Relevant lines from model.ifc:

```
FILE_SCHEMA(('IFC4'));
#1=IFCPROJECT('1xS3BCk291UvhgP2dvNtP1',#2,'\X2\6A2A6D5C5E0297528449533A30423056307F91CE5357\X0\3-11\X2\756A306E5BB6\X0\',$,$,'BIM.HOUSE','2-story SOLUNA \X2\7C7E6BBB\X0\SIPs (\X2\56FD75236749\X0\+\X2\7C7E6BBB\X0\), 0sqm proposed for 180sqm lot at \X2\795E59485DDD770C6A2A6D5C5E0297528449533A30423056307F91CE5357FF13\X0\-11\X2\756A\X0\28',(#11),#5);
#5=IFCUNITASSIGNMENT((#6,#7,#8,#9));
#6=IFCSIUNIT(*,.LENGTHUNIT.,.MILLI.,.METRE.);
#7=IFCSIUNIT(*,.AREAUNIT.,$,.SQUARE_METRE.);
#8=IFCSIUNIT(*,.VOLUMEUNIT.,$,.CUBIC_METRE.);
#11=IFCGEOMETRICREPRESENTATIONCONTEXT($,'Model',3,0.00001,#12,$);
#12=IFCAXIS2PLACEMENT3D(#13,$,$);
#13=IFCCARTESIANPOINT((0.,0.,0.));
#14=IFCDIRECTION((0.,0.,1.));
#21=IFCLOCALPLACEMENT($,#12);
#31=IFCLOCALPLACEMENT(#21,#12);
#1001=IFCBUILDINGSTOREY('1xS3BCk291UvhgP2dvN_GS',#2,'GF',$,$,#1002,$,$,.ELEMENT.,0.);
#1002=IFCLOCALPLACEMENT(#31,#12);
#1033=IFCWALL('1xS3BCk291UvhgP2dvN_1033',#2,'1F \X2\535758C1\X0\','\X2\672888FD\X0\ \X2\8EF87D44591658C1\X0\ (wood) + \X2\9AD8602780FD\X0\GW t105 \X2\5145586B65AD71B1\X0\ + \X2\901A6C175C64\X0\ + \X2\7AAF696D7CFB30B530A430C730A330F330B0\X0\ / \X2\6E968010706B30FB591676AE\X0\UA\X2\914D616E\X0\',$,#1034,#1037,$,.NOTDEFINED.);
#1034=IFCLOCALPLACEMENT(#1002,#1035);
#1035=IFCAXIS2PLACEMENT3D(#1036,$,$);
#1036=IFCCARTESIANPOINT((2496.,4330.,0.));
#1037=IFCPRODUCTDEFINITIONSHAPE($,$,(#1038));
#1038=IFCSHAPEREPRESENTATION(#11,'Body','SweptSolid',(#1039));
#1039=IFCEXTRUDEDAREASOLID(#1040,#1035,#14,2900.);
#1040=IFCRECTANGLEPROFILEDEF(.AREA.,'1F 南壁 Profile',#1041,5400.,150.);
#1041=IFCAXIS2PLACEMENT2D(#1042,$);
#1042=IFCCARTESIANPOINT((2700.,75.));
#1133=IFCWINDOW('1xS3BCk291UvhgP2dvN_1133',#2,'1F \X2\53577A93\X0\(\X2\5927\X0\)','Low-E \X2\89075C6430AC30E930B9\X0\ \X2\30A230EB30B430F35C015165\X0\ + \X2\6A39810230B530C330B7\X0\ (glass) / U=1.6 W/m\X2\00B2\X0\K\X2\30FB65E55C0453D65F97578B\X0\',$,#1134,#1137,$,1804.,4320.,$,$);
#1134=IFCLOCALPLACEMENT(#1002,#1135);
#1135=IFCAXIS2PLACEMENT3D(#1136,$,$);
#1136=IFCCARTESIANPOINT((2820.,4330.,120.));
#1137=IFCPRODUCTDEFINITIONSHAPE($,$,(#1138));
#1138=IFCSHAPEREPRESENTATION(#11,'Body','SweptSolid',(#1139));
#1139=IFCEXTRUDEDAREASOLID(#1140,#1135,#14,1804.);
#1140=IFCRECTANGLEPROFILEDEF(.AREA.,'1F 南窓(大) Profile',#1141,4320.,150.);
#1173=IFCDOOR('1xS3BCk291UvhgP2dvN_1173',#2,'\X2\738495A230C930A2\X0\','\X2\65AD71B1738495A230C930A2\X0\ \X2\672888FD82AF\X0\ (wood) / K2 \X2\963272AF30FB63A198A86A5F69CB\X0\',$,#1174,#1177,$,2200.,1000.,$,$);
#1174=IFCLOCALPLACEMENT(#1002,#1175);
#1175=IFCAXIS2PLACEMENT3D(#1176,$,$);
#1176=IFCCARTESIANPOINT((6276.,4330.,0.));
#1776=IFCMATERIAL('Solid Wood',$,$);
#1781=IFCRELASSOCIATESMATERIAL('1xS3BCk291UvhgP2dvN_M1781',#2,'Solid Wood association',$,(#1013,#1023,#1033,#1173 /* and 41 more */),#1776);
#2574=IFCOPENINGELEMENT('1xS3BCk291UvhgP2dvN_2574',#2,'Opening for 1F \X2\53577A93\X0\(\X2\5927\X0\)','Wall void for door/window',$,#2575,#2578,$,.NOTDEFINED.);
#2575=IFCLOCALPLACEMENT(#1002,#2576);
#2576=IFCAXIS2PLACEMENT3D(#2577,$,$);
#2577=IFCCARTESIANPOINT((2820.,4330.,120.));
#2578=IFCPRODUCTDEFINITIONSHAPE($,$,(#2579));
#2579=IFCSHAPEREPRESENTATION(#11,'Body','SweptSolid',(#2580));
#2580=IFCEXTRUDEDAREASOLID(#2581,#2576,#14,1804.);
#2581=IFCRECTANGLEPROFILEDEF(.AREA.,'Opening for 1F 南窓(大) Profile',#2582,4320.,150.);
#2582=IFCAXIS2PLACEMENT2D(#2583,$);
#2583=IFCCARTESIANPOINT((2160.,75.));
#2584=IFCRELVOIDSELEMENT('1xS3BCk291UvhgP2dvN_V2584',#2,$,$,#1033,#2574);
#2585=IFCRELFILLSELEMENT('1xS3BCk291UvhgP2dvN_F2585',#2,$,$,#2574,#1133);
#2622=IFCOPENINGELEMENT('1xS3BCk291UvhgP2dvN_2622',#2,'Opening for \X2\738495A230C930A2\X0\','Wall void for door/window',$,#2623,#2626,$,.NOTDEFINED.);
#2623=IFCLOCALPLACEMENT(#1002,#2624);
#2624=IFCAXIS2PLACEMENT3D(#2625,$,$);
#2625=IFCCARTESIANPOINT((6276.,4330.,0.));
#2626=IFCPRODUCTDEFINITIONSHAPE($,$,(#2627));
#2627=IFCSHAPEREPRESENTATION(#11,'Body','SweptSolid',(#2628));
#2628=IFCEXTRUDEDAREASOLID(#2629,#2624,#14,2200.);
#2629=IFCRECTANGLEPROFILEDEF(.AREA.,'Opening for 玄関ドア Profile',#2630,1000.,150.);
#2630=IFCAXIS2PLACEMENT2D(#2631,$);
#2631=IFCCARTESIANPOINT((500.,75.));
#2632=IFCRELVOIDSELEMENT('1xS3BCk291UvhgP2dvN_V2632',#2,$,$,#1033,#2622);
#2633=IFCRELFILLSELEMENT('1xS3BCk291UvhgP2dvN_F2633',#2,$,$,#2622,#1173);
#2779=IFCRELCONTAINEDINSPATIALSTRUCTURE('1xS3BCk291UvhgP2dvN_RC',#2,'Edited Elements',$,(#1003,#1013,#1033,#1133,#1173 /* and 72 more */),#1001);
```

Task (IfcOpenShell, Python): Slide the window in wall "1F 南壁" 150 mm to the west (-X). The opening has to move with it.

```python
import ifcopenshell
import ifcopenshell.api.geometry
import ifcopenshell.util.placement
import ifcopenshell.util.unit

model = ifcopenshell.open("model.ifc")
unit_scale = ifcopenshell.util.unit.calculate_unit_scale(model)

window = model.by_guid("1xS3BCk291UvhgP2dvN_1133")
opening = window.FillsVoids[0].RelatingOpeningElement
wall = opening.VoidsElements[0].RelatingBuildingElement

wall_matrix = ifcopenshell.util.placement.get_local_placement(wall.ObjectPlacement)
shift = wall_matrix[:3, 0] * -0.15 / unit_scale
before = ifcopenshell.util.placement.get_local_placement(window.ObjectPlacement)[:3, 3].copy()

# The window is not placed relative to its opening, so move both.
for product in (opening, window):
    matrix = ifcopenshell.util.placement.get_local_placement(product.ObjectPlacement)
    matrix[:3, 3] += shift
    ifcopenshell.api.geometry.edit_object_placement(model, product=product, matrix=matrix, is_si=False)

after = ifcopenshell.util.placement.get_local_placement(window.ObjectPlacement)[:3, 3]
print("window moved by", (after - before).round(3) + 0.0)

model.write("model_v2.ifc")
```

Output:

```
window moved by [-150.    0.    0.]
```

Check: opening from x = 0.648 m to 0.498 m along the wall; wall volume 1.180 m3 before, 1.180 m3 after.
